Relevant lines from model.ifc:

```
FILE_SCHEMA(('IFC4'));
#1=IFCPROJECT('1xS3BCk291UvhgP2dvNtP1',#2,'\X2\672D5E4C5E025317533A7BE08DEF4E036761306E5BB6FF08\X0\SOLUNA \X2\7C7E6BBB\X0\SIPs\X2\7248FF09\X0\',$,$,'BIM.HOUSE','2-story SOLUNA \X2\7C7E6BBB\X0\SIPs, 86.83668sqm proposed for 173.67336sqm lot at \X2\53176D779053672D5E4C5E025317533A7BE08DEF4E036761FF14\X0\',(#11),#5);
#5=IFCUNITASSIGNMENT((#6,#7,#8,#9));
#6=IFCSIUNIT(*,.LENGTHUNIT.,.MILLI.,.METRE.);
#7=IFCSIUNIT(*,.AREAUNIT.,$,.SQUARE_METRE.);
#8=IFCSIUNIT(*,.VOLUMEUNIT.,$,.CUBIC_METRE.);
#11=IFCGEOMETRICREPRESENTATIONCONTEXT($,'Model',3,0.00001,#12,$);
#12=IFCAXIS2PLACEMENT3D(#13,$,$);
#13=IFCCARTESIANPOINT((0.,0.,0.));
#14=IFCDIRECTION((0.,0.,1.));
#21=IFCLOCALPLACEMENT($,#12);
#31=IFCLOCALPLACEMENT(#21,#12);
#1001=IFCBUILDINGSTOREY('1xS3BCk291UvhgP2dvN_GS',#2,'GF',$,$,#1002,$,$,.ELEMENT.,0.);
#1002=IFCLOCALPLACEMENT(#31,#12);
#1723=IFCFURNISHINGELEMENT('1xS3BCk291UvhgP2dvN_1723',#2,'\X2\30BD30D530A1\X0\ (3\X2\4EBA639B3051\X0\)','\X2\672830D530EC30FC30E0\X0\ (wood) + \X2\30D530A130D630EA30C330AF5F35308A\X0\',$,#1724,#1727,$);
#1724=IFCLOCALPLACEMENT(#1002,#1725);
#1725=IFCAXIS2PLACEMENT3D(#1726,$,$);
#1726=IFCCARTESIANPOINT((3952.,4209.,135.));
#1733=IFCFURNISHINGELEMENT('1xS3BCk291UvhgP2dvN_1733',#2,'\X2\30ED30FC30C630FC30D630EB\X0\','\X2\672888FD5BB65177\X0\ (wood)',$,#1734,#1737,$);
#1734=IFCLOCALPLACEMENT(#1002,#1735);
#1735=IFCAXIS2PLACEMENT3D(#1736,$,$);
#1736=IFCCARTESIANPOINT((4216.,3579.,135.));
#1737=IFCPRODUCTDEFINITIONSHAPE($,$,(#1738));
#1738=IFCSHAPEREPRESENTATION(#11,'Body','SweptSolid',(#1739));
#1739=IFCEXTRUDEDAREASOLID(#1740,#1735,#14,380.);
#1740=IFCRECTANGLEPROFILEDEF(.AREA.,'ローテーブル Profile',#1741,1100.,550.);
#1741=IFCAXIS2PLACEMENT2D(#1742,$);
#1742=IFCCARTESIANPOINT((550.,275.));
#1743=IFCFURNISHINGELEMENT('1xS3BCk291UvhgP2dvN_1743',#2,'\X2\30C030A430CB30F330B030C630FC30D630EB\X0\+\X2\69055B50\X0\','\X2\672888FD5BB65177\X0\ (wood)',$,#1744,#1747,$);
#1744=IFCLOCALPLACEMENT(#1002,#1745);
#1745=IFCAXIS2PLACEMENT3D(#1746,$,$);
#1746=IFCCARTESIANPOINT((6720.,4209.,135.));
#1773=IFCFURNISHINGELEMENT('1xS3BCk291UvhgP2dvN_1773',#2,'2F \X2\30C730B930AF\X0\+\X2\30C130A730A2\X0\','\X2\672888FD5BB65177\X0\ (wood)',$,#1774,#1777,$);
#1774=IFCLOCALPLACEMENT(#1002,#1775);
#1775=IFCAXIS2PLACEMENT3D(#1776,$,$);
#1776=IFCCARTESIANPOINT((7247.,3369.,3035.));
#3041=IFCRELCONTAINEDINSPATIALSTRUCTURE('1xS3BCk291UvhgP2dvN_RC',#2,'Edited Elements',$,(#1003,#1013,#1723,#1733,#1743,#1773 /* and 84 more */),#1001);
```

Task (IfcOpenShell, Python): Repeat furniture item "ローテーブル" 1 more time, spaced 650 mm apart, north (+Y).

```python
import numpy as np
import ifcopenshell
import ifcopenshell.api.geometry
import ifcopenshell.api.root
import ifcopenshell.util.element
import ifcopenshell.util.placement

model = ifcopenshell.open("model.ifc")


def reuse_history(source, copy):
    """copy_class also copies each property set's owner history, people and application; keep the originals."""
    for rel in copy.IsDefinedBy:
        if rel.is_a("IfcRelDefinesByProperties") and (history := rel.RelatingPropertyDefinition.OwnerHistory):
            rel.RelatingPropertyDefinition.OwnerHistory = source.OwnerHistory
            ifcopenshell.util.element.remove_deep2(model, history)


source = model.by_guid("1xS3BCk291UvhgP2dvN_1733")
base = ifcopenshell.util.placement.get_local_placement(source.ObjectPlacement)
step = np.array([0.0, 1.0, 0.0]) * 650.0

for i in range(1, 2):
    copy = ifcopenshell.api.root.copy_class(model, product=source)
    copy.Representation = ifcopenshell.util.element.copy_deep(
        model, source.Representation, exclude=["IfcGeometricRepresentationContext", "IfcRepresentationMap"]
    )
    reuse_history(source, copy)
    matrix = base.copy()
    matrix[:3, 3] += i * step
    print("added at", matrix[:3, 3].round(3) + 0.0)
    ifcopenshell.api.geometry.edit_object_placement(model, product=copy, matrix=matrix, is_si=False)

model.write("model_rev.ifc")
```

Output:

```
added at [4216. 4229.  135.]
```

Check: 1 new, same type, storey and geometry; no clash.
